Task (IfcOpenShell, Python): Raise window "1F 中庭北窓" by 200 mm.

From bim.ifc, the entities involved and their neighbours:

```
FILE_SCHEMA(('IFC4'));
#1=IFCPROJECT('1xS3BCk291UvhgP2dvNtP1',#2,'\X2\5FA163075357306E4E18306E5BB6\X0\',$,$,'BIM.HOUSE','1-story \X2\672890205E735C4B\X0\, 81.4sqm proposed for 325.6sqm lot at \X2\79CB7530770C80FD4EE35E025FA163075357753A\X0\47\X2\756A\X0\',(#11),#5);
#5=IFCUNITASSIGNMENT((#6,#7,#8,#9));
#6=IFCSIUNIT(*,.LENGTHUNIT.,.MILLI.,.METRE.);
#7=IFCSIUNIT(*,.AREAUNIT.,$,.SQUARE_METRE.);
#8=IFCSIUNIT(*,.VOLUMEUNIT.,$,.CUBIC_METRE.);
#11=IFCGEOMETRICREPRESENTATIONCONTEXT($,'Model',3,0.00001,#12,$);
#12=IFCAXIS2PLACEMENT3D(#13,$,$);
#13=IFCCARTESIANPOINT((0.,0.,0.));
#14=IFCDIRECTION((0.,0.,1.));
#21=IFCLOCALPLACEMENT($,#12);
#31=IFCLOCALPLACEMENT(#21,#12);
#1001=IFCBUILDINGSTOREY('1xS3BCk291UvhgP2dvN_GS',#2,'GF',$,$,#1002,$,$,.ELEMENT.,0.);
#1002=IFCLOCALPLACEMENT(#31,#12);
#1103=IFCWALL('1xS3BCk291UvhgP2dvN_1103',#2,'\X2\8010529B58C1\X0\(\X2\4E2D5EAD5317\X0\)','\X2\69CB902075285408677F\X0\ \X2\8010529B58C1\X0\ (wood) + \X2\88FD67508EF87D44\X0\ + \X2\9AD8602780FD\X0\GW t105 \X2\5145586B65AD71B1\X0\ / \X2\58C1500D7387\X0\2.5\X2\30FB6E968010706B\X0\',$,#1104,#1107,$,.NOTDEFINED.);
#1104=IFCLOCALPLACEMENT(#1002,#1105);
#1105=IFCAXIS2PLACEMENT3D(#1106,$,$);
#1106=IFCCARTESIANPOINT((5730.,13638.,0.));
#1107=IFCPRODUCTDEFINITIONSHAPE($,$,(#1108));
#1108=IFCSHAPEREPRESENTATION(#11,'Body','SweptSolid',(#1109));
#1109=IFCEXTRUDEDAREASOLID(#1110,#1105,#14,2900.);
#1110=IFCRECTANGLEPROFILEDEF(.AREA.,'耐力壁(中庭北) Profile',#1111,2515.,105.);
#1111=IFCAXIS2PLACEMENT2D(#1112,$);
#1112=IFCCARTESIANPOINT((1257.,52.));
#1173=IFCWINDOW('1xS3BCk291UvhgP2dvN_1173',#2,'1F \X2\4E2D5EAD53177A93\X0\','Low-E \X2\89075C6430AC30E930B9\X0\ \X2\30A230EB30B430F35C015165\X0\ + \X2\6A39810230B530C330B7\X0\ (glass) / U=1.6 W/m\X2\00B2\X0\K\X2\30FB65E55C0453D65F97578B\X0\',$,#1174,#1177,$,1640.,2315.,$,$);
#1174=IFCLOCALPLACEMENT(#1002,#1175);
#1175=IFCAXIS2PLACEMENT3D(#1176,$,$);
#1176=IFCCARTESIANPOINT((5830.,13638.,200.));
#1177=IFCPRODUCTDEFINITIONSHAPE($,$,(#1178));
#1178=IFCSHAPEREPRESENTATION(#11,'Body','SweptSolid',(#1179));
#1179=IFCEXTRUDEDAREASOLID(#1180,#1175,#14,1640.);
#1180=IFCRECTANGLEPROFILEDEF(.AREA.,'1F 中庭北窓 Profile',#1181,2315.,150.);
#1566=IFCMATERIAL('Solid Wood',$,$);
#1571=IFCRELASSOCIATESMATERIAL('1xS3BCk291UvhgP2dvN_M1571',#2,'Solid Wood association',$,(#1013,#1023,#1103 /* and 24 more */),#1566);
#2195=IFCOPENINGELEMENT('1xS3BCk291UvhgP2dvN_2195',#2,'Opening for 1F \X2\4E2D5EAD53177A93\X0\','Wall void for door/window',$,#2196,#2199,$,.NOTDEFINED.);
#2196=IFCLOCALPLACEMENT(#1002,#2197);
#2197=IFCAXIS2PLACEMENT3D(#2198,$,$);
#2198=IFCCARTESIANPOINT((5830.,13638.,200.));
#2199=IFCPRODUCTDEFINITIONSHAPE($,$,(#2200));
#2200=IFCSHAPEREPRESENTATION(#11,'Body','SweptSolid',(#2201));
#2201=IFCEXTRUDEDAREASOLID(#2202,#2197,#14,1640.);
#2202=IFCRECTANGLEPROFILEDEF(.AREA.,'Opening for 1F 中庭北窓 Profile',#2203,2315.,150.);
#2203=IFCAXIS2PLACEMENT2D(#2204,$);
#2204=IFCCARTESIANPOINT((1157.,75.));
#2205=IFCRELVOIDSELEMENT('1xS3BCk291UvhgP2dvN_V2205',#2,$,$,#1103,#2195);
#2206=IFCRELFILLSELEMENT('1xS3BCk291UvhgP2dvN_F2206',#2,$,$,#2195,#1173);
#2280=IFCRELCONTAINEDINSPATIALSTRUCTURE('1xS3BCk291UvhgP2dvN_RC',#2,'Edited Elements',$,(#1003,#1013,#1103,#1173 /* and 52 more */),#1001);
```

```python
import numpy as np
import ifcopenshell
import ifcopenshell.api.geometry
import ifcopenshell.util.placement
import ifcopenshell.util.unit

model = ifcopenshell.open("bim.ifc")
unit_scale = ifcopenshell.util.unit.calculate_unit_scale(model)

window = model.by_guid("1xS3BCk291UvhgP2dvN_1173")
opening = window.FillsVoids[0].RelatingOpeningElement
dz = 200.0

shift = np.array([0.0, 0.0, dz])
# The window is not placed relative to its opening, so move both.
for product in (opening, window):
    matrix = ifcopenshell.util.placement.get_local_placement(product.ObjectPlacement)
    matrix[:3, 3] += shift
    ifcopenshell.api.geometry.edit_object_placement(model, product=product, matrix=matrix, is_si=False)

print(f"moved by {dz * unit_scale:+.3f} m")

model.write("bim_edited.ifc")
```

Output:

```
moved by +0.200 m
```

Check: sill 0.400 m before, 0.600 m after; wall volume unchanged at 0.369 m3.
